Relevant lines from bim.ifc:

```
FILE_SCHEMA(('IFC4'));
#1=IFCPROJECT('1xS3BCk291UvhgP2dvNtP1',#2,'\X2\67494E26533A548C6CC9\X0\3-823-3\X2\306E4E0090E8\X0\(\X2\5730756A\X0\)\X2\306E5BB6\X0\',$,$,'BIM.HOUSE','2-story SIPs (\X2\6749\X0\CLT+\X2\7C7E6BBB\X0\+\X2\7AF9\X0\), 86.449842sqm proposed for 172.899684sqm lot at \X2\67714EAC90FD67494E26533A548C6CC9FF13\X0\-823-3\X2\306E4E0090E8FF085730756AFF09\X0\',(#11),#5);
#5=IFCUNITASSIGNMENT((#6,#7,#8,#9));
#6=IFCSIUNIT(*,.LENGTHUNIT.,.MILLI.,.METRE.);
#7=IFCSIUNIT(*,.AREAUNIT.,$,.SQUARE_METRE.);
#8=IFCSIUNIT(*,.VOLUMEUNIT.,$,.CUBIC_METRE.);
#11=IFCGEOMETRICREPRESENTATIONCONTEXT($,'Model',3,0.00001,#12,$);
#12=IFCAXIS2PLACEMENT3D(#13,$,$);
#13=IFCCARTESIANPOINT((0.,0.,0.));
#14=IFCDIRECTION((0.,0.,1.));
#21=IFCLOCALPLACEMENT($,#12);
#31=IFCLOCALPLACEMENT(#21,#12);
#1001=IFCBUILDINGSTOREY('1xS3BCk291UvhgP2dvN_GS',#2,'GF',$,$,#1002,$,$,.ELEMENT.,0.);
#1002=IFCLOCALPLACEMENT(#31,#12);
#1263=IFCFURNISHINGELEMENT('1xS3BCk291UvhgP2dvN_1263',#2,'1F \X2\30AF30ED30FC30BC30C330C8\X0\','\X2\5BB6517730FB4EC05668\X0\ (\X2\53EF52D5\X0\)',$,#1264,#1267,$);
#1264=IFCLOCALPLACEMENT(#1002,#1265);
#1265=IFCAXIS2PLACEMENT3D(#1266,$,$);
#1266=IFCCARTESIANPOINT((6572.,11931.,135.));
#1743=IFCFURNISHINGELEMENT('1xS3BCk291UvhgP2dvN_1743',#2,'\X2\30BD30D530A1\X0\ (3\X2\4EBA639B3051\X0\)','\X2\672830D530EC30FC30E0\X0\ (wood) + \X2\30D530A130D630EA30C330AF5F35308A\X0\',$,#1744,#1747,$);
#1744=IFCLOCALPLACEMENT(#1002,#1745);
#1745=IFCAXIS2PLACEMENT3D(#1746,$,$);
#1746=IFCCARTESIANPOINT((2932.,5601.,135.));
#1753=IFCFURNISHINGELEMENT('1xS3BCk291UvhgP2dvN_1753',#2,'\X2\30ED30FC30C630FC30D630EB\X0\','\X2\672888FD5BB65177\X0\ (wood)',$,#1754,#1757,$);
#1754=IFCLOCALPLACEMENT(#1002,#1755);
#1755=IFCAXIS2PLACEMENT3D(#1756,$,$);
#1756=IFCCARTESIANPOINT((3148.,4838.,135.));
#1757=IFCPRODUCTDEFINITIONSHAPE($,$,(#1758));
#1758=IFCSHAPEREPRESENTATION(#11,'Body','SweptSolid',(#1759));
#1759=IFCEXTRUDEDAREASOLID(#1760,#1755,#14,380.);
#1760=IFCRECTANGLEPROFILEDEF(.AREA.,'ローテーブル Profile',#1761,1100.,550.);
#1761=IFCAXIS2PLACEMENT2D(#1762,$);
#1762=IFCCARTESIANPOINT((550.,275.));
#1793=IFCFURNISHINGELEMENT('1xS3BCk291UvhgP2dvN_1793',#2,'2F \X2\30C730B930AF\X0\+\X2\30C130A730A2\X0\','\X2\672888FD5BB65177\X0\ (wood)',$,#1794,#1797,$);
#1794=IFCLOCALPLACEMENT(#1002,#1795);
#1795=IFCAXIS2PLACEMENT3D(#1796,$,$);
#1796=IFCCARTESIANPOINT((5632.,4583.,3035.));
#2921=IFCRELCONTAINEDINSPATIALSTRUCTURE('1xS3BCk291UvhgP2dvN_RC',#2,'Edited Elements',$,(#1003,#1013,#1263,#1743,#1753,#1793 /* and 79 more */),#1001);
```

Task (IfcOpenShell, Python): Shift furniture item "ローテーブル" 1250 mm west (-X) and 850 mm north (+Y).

```python
import ifcopenshell
import ifcopenshell.api.geometry
import ifcopenshell.util.placement

model = ifcopenshell.open("bim.ifc")

item = model.by_guid("1xS3BCk291UvhgP2dvN_1753")
matrix = ifcopenshell.util.placement.get_local_placement(item.ObjectPlacement)
matrix[0, 3] -= 1250.0
matrix[1, 3] += 850.0
ifcopenshell.api.geometry.edit_object_placement(model, product=item, matrix=matrix, is_si=False)

print(ifcopenshell.util.placement.get_local_placement(item.ObjectPlacement).round(3) + 0.0)

model.write("bim_edited.ifc")
```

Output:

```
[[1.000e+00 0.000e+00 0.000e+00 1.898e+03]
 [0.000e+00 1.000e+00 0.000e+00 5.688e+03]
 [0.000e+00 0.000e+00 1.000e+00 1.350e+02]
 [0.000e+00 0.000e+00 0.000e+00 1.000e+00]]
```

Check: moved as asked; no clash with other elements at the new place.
